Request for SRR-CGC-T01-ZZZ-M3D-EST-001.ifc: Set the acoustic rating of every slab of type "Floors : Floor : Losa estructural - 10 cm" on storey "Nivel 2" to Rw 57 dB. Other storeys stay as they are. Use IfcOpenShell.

First a look at what the model holds.

```python
import ifcopenshell
import ifcopenshell.util.element

model = ifcopenshell.open("SRR-CGC-T01-ZZZ-M3D-EST-001.ifc")
print(model.schema)
storey = next(s for s in model.by_type("IfcBuildingStorey") if s.Name == "Nivel 2")
slabs = [e for e in ifcopenshell.util.element.get_decomposition(storey) if e.is_a("IfcSlab")]
seen = {}
for e in slabs:
    element_type = ifcopenshell.util.element.get_type(e)
    key = (element_type.Name if element_type != e and element_type else None, ifcopenshell.util.element.get_pset(e, "Pset_SlabCommon", "AcousticRating"))
    seen[key] = seen.get(key, 0) + 1
for (name, value), count in sorted(seen.items(), key=str):
    print(count, "x", name, "|", value)
```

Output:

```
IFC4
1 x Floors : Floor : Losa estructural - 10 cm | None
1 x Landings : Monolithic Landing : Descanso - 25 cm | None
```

```python
import ifcopenshell
import ifcopenshell.api.pset
import ifcopenshell.util.element

model = ifcopenshell.open("SRR-CGC-T01-ZZZ-M3D-EST-001.ifc")

storey = next(s for s in model.by_type("IfcBuildingStorey") if s.Name == "Nivel 2")
slabs = [e for e in ifcopenshell.util.element.get_decomposition(storey) if e.is_a("IfcSlab")]

count = 0
for e in slabs:
    element_type = ifcopenshell.util.element.get_type(e)
    if element_type in (None, e) or element_type.Name != "Floors : Floor : Losa estructural - 10 cm":
        continue
    # add_pset returns the element's existing set when there is one.
    pset = ifcopenshell.api.pset.add_pset(model, product=e, name="Pset_SlabCommon")
    ifcopenshell.api.pset.edit_pset(model, pset=pset, properties={"AcousticRating": "Rw 57 dB"})
    count += 1

print(count, "slabs updated")

model.write("SRR-CGC-T01-ZZZ-M3D-EST-001_edited.ifc")
```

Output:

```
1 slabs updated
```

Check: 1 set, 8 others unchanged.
